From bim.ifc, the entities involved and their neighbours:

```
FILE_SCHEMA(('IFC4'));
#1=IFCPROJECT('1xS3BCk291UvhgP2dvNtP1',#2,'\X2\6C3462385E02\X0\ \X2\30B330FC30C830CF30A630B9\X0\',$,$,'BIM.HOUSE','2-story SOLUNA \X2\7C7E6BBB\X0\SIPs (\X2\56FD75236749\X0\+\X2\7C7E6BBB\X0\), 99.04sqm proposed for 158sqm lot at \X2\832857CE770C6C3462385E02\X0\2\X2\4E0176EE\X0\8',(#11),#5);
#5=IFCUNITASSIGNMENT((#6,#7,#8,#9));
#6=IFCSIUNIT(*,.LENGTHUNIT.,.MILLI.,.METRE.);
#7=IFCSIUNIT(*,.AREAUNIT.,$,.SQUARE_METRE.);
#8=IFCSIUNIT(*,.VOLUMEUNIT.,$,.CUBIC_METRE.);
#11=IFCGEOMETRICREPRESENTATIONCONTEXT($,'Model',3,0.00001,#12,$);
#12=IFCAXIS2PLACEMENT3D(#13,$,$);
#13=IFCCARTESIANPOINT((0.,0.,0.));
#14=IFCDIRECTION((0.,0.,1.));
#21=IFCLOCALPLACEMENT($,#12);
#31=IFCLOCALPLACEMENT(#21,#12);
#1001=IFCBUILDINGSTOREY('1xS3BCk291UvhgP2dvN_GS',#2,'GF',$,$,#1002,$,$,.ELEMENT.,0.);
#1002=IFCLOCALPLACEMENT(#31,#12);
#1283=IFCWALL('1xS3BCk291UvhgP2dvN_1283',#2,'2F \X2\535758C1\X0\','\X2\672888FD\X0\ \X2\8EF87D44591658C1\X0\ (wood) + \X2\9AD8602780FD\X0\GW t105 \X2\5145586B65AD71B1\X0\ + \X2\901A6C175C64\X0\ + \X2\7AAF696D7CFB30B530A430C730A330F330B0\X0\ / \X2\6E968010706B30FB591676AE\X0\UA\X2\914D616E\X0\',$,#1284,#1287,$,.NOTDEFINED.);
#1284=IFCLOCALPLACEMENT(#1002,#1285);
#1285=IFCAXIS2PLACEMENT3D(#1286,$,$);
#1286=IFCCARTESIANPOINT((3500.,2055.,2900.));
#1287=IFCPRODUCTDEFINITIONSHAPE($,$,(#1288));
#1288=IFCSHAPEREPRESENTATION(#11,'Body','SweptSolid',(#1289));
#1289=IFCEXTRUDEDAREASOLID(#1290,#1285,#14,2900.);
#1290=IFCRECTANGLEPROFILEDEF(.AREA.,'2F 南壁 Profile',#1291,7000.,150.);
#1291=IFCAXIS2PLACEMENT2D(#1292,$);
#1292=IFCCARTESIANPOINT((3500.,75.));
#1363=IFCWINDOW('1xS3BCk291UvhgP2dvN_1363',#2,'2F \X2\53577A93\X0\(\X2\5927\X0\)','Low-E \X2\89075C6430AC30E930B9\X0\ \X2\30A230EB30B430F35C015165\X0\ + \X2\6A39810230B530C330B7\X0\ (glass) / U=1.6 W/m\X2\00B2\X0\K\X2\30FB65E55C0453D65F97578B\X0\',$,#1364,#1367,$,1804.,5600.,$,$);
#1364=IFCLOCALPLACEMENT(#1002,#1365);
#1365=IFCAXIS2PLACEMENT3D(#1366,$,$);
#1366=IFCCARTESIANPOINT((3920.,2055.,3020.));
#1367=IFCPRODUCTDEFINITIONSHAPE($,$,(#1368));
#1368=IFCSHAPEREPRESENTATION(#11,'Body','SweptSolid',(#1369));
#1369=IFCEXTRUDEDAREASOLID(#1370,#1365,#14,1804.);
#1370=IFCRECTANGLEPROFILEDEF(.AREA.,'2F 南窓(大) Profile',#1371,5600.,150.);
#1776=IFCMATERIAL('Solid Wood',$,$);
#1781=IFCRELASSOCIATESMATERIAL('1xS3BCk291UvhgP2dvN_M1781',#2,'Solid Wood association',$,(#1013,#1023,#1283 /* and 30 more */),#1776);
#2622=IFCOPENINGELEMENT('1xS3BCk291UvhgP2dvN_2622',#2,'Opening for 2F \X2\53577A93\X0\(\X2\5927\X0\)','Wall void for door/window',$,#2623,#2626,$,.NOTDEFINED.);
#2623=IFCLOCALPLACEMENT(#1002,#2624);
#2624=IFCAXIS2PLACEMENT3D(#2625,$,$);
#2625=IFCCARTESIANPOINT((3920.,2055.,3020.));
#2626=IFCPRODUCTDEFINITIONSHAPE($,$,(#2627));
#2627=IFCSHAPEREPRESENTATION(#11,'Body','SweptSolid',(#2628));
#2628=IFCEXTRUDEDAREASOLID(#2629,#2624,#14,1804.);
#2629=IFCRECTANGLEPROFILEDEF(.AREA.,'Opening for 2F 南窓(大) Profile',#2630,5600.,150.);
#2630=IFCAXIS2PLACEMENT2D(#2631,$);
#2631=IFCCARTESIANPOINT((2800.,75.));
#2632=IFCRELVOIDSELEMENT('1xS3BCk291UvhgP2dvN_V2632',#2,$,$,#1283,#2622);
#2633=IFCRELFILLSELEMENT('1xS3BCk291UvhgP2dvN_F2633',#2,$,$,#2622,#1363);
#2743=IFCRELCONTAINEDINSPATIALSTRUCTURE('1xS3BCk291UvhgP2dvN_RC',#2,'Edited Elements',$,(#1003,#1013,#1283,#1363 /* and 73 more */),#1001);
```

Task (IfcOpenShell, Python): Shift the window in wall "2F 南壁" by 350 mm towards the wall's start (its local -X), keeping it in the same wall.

```python
import ifcopenshell
import ifcopenshell.api.geometry
import ifcopenshell.util.placement
import ifcopenshell.util.unit

model = ifcopenshell.open("bim.ifc")
unit_scale = ifcopenshell.util.unit.calculate_unit_scale(model)

window = model.by_guid("1xS3BCk291UvhgP2dvN_1363")
opening = window.FillsVoids[0].RelatingOpeningElement
wall = opening.VoidsElements[0].RelatingBuildingElement

wall_matrix = ifcopenshell.util.placement.get_local_placement(wall.ObjectPlacement)
shift = wall_matrix[:3, 0] * -0.35 / unit_scale
before = ifcopenshell.util.placement.get_local_placement(window.ObjectPlacement)[:3, 3].copy()

# The window is not placed relative to its opening, so move both.
for product in (opening, window):
    matrix = ifcopenshell.util.placement.get_local_placement(product.ObjectPlacement)
    matrix[:3, 3] += shift
    ifcopenshell.api.geometry.edit_object_placement(model, product=product, matrix=matrix, is_si=False)

after = ifcopenshell.util.placement.get_local_placement(window.ObjectPlacement)[:3, 3]
print("window moved by", (after - before).round(3) + 0.0)

model.write("bim_rev.ifc")
```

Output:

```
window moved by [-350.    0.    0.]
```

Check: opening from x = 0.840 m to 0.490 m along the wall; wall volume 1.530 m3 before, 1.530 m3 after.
